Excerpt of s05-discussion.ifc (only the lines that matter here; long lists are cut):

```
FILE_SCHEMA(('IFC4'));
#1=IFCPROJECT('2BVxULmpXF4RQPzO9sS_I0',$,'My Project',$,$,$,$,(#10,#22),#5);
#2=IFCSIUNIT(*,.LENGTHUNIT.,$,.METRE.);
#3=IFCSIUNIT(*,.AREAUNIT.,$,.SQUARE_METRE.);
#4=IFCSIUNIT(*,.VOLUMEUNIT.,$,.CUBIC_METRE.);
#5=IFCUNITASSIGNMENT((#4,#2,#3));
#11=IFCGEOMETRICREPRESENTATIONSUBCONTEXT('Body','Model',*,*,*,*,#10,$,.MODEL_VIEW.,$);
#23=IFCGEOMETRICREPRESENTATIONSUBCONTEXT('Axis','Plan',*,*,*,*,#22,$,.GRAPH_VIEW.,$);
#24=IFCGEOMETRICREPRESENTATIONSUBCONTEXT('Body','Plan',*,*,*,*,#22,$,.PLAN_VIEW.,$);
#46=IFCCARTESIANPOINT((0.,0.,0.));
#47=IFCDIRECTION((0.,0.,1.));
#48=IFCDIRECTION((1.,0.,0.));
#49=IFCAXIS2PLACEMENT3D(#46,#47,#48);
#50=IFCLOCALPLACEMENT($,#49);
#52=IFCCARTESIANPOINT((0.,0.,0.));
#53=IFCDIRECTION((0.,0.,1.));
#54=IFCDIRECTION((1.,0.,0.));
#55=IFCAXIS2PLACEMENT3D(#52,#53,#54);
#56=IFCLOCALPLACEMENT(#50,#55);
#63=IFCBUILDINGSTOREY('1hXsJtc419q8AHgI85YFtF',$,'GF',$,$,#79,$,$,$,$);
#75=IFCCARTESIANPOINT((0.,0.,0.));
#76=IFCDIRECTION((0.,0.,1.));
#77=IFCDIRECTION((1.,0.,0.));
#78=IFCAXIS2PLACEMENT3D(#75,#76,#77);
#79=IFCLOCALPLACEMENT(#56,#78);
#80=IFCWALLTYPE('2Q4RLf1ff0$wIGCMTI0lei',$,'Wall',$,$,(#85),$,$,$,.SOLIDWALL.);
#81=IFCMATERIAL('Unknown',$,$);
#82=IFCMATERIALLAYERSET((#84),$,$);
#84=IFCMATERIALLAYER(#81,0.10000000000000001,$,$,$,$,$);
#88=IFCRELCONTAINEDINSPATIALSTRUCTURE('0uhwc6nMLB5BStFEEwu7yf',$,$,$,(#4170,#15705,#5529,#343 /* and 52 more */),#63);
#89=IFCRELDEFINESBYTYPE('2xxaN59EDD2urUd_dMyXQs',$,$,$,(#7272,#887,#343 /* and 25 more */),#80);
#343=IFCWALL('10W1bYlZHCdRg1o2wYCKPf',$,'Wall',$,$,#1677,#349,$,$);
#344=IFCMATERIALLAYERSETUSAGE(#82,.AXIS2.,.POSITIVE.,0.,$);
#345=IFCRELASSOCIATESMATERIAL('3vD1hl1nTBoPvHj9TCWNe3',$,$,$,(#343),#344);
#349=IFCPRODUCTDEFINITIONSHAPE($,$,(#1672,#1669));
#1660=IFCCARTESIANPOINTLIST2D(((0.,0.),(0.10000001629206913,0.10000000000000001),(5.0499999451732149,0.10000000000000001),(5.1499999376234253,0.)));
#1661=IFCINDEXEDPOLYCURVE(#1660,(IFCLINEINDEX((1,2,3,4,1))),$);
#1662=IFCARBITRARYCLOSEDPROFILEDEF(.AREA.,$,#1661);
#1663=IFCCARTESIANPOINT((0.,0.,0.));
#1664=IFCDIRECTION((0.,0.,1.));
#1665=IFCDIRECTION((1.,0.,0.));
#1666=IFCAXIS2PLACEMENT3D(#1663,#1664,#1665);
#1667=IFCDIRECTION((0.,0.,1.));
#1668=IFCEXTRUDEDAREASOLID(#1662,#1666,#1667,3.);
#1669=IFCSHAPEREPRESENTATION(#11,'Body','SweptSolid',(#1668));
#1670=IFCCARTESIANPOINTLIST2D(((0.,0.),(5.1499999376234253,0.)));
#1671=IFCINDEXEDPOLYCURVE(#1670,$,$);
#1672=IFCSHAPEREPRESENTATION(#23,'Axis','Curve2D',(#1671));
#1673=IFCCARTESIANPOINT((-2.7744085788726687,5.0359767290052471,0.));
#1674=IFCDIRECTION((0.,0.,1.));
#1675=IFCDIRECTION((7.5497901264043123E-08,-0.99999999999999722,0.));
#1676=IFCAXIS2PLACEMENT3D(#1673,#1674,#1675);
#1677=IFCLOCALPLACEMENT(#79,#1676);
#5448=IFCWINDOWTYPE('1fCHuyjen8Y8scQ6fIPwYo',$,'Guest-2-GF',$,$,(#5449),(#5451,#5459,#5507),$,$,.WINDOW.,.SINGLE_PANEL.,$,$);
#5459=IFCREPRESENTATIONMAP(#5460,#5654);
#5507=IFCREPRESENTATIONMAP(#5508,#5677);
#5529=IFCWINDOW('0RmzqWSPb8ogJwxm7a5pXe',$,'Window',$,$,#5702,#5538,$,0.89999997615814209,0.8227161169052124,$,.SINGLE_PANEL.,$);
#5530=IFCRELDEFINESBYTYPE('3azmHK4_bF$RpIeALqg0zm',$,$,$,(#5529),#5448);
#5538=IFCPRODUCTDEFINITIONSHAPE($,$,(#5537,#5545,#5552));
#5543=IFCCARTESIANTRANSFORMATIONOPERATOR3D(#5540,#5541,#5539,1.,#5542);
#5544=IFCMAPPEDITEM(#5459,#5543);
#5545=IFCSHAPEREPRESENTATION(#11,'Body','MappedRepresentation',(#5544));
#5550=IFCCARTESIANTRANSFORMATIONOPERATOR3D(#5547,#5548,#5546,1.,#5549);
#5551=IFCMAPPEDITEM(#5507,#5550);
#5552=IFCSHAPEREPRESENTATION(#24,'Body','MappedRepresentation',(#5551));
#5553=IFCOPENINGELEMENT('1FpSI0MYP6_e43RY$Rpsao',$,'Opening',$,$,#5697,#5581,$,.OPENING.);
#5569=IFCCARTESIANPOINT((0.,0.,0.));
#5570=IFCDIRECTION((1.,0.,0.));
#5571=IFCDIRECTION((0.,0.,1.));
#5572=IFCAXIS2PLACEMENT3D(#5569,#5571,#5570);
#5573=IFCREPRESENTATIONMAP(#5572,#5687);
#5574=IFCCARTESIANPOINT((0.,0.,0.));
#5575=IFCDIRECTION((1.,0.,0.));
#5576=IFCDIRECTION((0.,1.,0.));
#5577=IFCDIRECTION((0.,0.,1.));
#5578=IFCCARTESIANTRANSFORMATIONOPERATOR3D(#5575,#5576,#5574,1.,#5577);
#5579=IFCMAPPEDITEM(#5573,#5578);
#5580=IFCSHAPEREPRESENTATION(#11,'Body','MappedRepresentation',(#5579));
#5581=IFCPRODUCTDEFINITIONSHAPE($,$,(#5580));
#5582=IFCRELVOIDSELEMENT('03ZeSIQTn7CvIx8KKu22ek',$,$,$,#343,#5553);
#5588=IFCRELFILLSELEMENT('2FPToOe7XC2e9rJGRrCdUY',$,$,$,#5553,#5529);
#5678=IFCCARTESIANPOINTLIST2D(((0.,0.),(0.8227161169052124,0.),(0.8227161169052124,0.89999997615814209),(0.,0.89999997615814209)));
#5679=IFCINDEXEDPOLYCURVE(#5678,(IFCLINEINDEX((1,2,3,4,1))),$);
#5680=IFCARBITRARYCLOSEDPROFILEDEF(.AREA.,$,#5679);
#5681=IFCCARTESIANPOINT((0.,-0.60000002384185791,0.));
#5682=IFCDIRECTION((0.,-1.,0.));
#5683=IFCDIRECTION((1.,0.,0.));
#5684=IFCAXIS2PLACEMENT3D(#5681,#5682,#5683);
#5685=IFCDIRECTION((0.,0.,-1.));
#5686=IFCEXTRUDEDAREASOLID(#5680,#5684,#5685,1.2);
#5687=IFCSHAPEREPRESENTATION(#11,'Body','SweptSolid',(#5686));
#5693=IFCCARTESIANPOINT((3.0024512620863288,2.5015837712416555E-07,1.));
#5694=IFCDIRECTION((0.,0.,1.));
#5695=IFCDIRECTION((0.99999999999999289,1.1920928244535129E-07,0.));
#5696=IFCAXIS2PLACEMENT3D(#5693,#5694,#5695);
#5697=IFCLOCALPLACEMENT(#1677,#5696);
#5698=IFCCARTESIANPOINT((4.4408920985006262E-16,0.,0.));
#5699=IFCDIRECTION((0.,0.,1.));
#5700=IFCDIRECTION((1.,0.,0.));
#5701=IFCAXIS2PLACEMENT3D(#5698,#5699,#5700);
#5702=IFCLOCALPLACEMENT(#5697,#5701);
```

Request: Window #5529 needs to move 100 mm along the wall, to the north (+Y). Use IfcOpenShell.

```python
import ifcopenshell
import ifcopenshell.api.geometry
import ifcopenshell.util.placement

model = ifcopenshell.open("s05-discussion.ifc")

window = model.by_guid("0RmzqWSPb8ogJwxm7a5pXe")
opening = window.FillsVoids[0].RelatingOpeningElement
wall = opening.VoidsElements[0].RelatingBuildingElement

wall_matrix = ifcopenshell.util.placement.get_local_placement(wall.ObjectPlacement)
shift = wall_matrix[:3, 0] * -0.1
before = ifcopenshell.util.placement.get_local_placement(window.ObjectPlacement)[:3, 3].copy()

# The window is placed relative to its opening, so it follows when the opening moves.
matrix = ifcopenshell.util.placement.get_local_placement(opening.ObjectPlacement)
matrix[:3, 3] += shift
ifcopenshell.api.geometry.edit_object_placement(
    model, product=opening, matrix=matrix, is_si=False, should_transform_children=True
)

after = ifcopenshell.util.placement.get_local_placement(window.ObjectPlacement)[:3, 3]
print("window moved by", (after - before).round(3) + 0.0)

model.write("s05-discussion_updated.ifc")
```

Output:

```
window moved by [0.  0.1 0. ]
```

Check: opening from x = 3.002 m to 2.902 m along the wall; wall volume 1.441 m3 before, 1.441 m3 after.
